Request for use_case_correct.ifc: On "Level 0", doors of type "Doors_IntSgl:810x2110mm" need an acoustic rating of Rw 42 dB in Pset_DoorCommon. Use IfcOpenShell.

First a look at what the model holds.

```python
import ifcopenshell
import ifcopenshell.util.element

model = ifcopenshell.open("use_case_correct.ifc")
print(model.schema)
storey = next(s for s in model.by_type("IfcBuildingStorey") if s.Name == "Level 0")
doors = [e for e in ifcopenshell.util.element.get_decomposition(storey) if e.is_a("IfcDoor")]
seen = {}
for e in doors:
    element_type = ifcopenshell.util.element.get_type(e)
    key = (element_type.Name if element_type != e and element_type else None, ifcopenshell.util.element.get_pset(e, "Pset_DoorCommon", "AcousticRating"))
    seen[key] = seen.get(key, 0) + 1
for (name, value), count in sorted(seen.items(), key=str):
    print(count, "x", name, "|", value)
```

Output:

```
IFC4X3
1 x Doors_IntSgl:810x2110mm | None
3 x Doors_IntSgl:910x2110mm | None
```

```python
import ifcopenshell
import ifcopenshell.api.pset
import ifcopenshell.util.element

model = ifcopenshell.open("use_case_correct.ifc")

storey = next(s for s in model.by_type("IfcBuildingStorey") if s.Name == "Level 0")
doors = [e for e in ifcopenshell.util.element.get_decomposition(storey) if e.is_a("IfcDoor")]

count = 0
for e in doors:
    element_type = ifcopenshell.util.element.get_type(e)
    if element_type in (None, e) or element_type.Name != "Doors_IntSgl:810x2110mm":
        continue
    # add_pset returns the element's existing set when there is one.
    pset = ifcopenshell.api.pset.add_pset(model, product=e, name="Pset_DoorCommon")
    ifcopenshell.api.pset.edit_pset(model, pset=pset, properties={"AcousticRating": "Rw 42 dB"})
    count += 1

print(count, "doors updated")

model.write("use_case_correct_updated.ifc")
```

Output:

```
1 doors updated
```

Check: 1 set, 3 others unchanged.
